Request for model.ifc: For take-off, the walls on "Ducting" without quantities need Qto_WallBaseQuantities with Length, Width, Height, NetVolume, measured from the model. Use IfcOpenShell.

First a look at what the model holds.

```python
import ifcopenshell
import ifcopenshell.util.element
import ifcopenshell.util.unit

model = ifcopenshell.open("model.ifc")
print(model.schema)
for unit_type in ("LENGTHUNIT", "AREAUNIT", "VOLUMEUNIT"):
    print(unit_type, ifcopenshell.util.unit.calculate_unit_scale(model, unit_type))
storey = next(s for s in model.by_type("IfcBuildingStorey") if s.Name == "Ducting")
walls = [e for e in ifcopenshell.util.element.get_decomposition(storey) if e.is_a("IfcWall")]
for e in sorted(walls, key=lambda e: e.id()):
    print(e.id(), e.is_a(), e.Name, list(ifcopenshell.util.element.get_psets(e, qtos_only=True)), sep=" | ")
```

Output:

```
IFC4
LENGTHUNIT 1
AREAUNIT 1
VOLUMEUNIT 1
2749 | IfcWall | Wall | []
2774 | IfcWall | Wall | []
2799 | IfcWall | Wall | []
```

```python
import ifcopenshell
import ifcopenshell.api.pset
import ifcopenshell.geom
import ifcopenshell.util.element
import ifcopenshell.util.shape
import ifcopenshell.util.unit

model = ifcopenshell.open("model.ifc")
unit_scale = ifcopenshell.util.unit.calculate_unit_scale(model)
volume_scale = ifcopenshell.util.unit.calculate_unit_scale(model, "VOLUMEUNIT")
settings = ifcopenshell.geom.settings()

storey = next(s for s in model.by_type("IfcBuildingStorey") if s.Name == "Ducting")
walls = [e for e in ifcopenshell.util.element.get_decomposition(storey) if e.is_a("IfcWall")]

for e in sorted(walls, key=lambda e: e.id()):
    if ifcopenshell.util.element.get_psets(e, qtos_only=True, should_inherit=False):
        continue
    # Geometry comes back in metres, in the element's own axes.
    shape = ifcopenshell.geom.create_shape(settings, e)
    values = {
        "Length": ifcopenshell.util.shape.get_x(shape.geometry) / unit_scale,
        "Width": ifcopenshell.util.shape.get_y(shape.geometry) / unit_scale,
        "Height": ifcopenshell.util.shape.get_z(shape.geometry) / unit_scale,
        "NetVolume": ifcopenshell.util.shape.get_volume(shape.geometry) / volume_scale,
    }
    qto = ifcopenshell.api.pset.add_qto(model, product=e, name="Qto_WallBaseQuantities")
    ifcopenshell.api.pset.edit_qto(model, qto=qto, properties=values)
    print(e.id(), {k: round(v, 3) for k, v in values.items()})

model.write("model_rev.ifc")
```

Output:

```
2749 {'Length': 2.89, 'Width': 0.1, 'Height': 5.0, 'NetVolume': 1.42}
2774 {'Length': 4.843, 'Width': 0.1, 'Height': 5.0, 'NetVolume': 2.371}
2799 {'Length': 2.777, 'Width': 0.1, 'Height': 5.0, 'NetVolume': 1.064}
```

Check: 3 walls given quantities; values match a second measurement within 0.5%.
